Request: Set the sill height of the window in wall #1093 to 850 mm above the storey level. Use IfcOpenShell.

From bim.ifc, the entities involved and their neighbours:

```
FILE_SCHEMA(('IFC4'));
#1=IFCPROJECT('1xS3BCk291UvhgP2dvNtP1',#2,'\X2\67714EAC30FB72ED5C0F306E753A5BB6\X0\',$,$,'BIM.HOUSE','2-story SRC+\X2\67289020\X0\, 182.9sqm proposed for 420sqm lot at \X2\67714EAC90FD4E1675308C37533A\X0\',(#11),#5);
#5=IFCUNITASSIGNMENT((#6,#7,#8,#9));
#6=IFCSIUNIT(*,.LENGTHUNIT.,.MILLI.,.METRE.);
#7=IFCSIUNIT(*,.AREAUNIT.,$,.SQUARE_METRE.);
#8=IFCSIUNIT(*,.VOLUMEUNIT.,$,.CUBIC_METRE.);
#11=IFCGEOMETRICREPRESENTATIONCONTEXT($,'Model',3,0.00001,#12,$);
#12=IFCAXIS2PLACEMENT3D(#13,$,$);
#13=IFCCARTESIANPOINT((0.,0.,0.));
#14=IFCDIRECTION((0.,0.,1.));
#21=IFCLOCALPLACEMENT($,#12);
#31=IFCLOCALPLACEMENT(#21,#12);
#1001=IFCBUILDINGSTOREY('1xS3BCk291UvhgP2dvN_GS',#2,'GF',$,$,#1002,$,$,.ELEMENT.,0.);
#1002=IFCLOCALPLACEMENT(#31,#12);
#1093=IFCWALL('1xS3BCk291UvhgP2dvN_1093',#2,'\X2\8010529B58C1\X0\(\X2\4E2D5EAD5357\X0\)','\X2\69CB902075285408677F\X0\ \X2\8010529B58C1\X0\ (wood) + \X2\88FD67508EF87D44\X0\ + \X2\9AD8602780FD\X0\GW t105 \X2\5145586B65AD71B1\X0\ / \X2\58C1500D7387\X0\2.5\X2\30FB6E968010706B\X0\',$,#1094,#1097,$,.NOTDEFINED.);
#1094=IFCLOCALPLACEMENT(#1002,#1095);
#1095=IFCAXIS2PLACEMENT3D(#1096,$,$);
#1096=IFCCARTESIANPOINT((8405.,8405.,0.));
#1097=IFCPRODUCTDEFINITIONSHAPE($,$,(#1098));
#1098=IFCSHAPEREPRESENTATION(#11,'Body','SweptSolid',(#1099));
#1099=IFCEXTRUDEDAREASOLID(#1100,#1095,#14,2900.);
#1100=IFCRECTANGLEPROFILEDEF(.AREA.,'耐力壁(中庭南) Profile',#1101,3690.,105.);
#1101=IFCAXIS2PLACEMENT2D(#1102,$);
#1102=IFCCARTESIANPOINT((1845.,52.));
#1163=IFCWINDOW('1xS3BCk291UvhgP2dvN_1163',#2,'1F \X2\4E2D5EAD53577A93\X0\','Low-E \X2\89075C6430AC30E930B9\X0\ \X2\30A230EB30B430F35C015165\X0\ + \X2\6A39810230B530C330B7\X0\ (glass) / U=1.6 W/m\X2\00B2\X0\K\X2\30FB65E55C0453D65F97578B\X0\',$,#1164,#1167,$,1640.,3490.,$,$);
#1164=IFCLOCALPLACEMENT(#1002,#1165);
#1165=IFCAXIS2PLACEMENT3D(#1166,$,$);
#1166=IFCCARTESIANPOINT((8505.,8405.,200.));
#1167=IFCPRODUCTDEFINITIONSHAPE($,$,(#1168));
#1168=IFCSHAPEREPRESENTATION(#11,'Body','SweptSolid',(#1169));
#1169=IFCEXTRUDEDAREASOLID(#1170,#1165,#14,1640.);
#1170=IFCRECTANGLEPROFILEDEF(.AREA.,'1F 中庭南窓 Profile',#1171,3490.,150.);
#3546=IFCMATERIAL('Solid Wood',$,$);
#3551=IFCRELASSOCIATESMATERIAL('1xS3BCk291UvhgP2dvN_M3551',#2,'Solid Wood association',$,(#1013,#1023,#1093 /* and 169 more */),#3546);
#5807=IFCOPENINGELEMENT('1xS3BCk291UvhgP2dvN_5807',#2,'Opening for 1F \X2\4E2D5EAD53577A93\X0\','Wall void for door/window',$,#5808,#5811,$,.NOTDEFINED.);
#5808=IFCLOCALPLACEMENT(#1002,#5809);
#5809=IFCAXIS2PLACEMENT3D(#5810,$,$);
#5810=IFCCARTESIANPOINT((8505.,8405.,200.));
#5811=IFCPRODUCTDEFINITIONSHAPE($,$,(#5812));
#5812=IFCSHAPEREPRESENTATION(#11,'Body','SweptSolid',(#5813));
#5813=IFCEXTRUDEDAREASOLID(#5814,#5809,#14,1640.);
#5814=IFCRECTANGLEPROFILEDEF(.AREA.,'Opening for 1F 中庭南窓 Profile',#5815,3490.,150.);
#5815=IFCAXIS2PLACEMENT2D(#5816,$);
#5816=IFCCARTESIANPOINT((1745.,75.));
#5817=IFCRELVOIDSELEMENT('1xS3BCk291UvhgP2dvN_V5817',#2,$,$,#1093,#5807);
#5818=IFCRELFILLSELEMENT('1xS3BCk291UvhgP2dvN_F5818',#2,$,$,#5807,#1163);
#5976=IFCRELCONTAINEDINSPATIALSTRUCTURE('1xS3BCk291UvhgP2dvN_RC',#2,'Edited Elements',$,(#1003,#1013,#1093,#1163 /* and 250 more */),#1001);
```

```python
import numpy as np
import ifcopenshell
import ifcopenshell.api.geometry
import ifcopenshell.geom
import ifcopenshell.util.element
import ifcopenshell.util.placement
import ifcopenshell.util.shape
import ifcopenshell.util.unit

model = ifcopenshell.open("bim.ifc")
unit_scale = ifcopenshell.util.unit.calculate_unit_scale(model)

window = model.by_guid("1xS3BCk291UvhgP2dvN_1163")
opening = window.FillsVoids[0].RelatingOpeningElement
storey = ifcopenshell.util.element.get_container(window, ifc_class="IfcBuildingStorey")
level = ifcopenshell.util.placement.get_local_placement(storey.ObjectPlacement)[2, 3]

# The opening's origin need not be at the sill, so measure its lowest point.
shape = ifcopenshell.geom.create_shape(ifcopenshell.geom.settings(), opening)
bottom = ifcopenshell.util.shape.get_shape_bottom_elevation(shape, shape.geometry) / unit_scale
dz = level + 850.0 - bottom

shift = np.array([0.0, 0.0, dz])
# The window is not placed relative to its opening, so move both.
for product in (opening, window):
    matrix = ifcopenshell.util.placement.get_local_placement(product.ObjectPlacement)
    matrix[:3, 3] += shift
    ifcopenshell.api.geometry.edit_object_placement(model, product=product, matrix=matrix, is_si=False)

print(f"moved by {dz * unit_scale:+.3f} m")

model.write("bim_edited.ifc")
```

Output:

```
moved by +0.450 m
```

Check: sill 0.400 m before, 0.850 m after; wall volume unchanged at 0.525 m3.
